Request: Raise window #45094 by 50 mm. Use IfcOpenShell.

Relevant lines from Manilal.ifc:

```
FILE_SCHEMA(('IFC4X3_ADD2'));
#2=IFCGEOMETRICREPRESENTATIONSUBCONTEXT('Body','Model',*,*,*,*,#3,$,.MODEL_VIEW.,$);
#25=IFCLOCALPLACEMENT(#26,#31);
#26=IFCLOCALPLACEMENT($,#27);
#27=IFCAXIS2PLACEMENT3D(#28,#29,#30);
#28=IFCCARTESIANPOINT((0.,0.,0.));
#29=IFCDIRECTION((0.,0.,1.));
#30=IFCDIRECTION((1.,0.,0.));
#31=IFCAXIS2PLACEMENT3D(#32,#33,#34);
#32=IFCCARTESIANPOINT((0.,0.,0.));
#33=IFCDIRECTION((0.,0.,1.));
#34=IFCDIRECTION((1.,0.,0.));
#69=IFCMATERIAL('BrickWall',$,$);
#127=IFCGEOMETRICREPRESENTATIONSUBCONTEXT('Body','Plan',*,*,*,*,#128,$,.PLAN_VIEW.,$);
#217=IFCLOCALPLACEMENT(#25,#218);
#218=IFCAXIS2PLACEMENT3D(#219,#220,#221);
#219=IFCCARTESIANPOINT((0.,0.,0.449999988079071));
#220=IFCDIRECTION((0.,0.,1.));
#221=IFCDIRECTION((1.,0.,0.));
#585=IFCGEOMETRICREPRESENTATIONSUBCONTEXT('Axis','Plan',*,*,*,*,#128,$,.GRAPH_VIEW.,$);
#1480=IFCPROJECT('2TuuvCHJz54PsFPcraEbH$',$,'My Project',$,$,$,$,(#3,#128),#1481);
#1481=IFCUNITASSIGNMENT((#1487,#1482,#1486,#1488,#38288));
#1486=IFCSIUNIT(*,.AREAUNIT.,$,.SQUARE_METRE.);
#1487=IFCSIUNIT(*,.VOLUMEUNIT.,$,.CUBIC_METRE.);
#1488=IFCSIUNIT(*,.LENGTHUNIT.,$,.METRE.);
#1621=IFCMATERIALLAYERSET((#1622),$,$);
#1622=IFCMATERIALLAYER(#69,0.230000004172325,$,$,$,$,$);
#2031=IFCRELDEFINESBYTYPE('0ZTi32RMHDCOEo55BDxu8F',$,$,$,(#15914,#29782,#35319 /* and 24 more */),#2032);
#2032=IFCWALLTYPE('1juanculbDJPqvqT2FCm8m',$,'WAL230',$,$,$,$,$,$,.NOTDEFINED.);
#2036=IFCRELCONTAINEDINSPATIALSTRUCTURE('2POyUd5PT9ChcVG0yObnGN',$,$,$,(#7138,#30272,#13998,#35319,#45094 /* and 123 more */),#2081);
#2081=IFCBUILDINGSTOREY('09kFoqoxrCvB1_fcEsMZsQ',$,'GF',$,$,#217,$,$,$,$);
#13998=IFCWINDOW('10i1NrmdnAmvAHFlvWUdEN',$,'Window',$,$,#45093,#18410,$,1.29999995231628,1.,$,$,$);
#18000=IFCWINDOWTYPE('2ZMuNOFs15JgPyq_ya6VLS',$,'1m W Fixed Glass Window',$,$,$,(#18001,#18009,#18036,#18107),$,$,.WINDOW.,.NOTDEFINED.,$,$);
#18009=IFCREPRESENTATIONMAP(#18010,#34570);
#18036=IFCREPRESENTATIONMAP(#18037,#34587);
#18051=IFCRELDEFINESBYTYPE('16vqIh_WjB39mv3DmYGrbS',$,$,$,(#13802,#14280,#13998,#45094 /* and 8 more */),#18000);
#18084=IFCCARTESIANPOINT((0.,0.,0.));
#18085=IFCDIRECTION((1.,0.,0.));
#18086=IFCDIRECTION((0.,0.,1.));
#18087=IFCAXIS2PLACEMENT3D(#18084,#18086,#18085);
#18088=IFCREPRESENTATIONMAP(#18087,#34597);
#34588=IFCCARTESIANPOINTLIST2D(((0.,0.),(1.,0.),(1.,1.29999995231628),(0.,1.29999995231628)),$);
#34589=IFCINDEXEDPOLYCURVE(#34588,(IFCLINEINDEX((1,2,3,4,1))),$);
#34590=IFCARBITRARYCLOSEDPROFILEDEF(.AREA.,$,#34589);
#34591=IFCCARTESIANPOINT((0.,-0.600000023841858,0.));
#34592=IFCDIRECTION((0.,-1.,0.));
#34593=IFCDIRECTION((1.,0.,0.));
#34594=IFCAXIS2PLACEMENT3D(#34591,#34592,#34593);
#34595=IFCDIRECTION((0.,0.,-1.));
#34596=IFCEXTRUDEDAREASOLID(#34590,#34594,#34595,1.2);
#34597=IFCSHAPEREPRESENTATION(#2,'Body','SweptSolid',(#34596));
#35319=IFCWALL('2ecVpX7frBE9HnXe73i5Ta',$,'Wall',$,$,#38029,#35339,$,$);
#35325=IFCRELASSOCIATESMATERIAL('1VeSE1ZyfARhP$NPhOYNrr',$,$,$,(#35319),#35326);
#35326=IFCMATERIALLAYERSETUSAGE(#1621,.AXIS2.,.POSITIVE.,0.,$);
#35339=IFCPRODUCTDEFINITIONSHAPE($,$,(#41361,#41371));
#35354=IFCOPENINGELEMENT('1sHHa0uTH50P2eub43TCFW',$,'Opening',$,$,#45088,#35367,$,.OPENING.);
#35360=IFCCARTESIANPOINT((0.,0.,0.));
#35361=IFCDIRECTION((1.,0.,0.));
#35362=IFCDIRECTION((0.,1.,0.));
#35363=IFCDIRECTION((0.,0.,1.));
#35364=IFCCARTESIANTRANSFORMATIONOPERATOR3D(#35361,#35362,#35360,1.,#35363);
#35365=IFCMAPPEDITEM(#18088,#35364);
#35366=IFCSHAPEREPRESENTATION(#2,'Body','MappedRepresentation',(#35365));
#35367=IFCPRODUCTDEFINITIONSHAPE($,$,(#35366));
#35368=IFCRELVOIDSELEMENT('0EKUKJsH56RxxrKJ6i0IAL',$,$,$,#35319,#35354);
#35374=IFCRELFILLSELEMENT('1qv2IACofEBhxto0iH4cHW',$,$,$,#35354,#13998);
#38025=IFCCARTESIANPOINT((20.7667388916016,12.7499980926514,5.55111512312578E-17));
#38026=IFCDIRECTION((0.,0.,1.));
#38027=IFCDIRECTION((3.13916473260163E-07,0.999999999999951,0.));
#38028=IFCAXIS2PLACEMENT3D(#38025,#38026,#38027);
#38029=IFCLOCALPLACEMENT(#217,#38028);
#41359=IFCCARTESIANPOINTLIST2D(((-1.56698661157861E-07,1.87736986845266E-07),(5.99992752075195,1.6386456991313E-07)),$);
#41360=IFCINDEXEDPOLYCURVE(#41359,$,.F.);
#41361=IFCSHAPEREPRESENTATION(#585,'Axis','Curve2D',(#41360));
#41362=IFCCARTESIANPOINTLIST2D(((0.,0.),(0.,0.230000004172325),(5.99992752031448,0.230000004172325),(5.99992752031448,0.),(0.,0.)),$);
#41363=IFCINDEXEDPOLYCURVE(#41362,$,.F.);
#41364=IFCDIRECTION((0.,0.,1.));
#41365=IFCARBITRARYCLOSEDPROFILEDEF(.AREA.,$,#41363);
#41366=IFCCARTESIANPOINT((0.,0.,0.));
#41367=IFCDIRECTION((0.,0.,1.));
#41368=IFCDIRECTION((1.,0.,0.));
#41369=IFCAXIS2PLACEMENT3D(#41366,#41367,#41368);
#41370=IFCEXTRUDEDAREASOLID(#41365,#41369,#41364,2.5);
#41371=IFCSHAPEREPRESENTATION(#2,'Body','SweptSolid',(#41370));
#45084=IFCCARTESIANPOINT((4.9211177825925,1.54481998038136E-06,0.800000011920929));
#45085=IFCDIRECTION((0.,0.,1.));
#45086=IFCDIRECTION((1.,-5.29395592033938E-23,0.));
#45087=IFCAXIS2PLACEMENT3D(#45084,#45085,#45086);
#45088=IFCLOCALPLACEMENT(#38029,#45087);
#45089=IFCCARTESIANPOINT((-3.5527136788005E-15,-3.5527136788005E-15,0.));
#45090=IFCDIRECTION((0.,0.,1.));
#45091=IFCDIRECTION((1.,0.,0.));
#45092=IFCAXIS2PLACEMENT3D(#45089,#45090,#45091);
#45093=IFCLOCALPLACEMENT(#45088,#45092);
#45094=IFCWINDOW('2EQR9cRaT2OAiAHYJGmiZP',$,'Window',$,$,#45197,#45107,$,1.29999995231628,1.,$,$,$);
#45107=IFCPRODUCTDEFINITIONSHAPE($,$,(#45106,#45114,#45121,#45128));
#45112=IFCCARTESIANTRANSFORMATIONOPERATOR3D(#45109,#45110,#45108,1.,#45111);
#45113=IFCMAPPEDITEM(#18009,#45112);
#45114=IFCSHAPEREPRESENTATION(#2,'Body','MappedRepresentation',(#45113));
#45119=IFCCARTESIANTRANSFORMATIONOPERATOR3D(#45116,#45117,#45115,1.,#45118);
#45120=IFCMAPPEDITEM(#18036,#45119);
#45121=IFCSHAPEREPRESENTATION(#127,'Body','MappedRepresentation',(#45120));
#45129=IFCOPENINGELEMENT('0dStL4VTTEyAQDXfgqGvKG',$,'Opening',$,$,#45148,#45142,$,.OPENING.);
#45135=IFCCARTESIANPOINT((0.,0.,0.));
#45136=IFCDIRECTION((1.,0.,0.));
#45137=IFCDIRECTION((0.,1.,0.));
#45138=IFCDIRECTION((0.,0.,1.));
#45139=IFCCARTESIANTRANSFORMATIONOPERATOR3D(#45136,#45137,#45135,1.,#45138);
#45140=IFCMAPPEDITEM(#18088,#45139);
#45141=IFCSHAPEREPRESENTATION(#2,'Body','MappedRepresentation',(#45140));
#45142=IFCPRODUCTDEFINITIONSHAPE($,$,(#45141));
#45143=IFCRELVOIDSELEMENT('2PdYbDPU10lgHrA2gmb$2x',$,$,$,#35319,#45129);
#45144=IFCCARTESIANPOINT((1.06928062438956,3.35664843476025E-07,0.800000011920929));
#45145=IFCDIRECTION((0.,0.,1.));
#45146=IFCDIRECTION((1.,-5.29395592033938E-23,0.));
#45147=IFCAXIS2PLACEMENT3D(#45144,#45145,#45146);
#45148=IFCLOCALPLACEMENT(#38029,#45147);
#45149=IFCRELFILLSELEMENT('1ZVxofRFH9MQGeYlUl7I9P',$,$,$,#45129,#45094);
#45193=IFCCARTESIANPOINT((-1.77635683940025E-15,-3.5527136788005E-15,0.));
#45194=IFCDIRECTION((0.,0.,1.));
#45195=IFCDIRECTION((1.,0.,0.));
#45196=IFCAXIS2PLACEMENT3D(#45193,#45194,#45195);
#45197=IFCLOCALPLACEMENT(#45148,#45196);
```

```python
import numpy as np
import ifcopenshell
import ifcopenshell.api.geometry
import ifcopenshell.util.placement
import ifcopenshell.util.unit

model = ifcopenshell.open("Manilal.ifc")
unit_scale = ifcopenshell.util.unit.calculate_unit_scale(model)

window = model.by_guid("2EQR9cRaT2OAiAHYJGmiZP")
opening = window.FillsVoids[0].RelatingOpeningElement
dz = 0.05

shift = np.array([0.0, 0.0, dz])
# The window is placed relative to its opening, so it follows when the opening moves.
matrix = ifcopenshell.util.placement.get_local_placement(opening.ObjectPlacement)
matrix[:3, 3] += shift
ifcopenshell.api.geometry.edit_object_placement(
    model, product=opening, matrix=matrix, is_si=False, should_transform_children=True
)

print(f"moved by {dz * unit_scale:+.3f} m")

model.write("Manilal_rev.ifc")
```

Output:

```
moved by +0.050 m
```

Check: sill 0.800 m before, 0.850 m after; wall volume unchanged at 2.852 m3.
